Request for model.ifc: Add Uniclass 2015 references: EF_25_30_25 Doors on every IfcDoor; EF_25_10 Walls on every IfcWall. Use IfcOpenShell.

First a look at what the model holds.

```python
import ifcopenshell

model = ifcopenshell.open("model.ifc")
print(model.schema)
print("classifications:", [c.Name for c in model.by_type("IfcClassification")])
for ifc_class in ("IfcDoor", "IfcRoof", "IfcStair", "IfcWall", "IfcWindow"):
    print(ifc_class, len(model.by_type(ifc_class)))
```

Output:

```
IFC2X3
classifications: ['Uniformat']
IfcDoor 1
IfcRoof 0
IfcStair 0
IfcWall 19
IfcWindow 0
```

```python
import ifcopenshell
import ifcopenshell.api.classification

model = ifcopenshell.open("model.ifc")

# IFC2X3 requires Source and Edition and has no link from the project to the system.
system = model.create_entity("IfcClassification", Source="NBS", Edition="2015", Name="Uniclass 2015")

codes = {
    "IfcDoor": ("EF_25_30_25", "Doors"),
    "IfcWall": ("EF_25_10", "Walls"),
}
for ifc_class, (code, name) in codes.items():
    products = model.by_type(ifc_class)
    ifcopenshell.api.classification.add_reference(
        model, products=products, classification=system, identification=code, name=name
    )
    print(code, len(products))

model.write("model_updated.ifc")
```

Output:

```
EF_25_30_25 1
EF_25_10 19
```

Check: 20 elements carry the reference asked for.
